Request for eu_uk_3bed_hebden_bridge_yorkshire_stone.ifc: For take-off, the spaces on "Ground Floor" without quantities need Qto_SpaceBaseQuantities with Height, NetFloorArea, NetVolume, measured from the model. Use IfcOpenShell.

First a look at what the model holds.

```python
import ifcopenshell
import ifcopenshell.util.element
import ifcopenshell.util.unit

model = ifcopenshell.open("eu_uk_3bed_hebden_bridge_yorkshire_stone.ifc")
print(model.schema)
for unit_type in ("LENGTHUNIT", "AREAUNIT", "VOLUMEUNIT"):
    print(unit_type, ifcopenshell.util.unit.calculate_unit_scale(model, unit_type))
storey = next(s for s in model.by_type("IfcBuildingStorey") if s.Name == "Ground Floor")
spaces = [e for e in ifcopenshell.util.element.get_decomposition(storey) if e.is_a("IfcSpace")]
for e in sorted(spaces, key=lambda e: e.id()):
    print(e.id(), e.is_a(), e.Name, list(ifcopenshell.util.element.get_psets(e, qtos_only=True)), sep=" | ")
```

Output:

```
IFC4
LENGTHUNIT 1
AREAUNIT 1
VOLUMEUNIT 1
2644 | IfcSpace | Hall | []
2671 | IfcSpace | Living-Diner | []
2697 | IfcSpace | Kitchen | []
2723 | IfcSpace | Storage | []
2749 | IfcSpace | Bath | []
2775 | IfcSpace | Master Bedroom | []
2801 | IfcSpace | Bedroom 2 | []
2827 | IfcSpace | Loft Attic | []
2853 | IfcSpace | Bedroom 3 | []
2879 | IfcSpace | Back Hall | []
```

```python
import ifcopenshell
import ifcopenshell.api.pset
import ifcopenshell.geom
import ifcopenshell.util.element
import ifcopenshell.util.shape
import ifcopenshell.util.unit

model = ifcopenshell.open("eu_uk_3bed_hebden_bridge_yorkshire_stone.ifc")
unit_scale = ifcopenshell.util.unit.calculate_unit_scale(model)
area_scale = ifcopenshell.util.unit.calculate_unit_scale(model, "AREAUNIT")
volume_scale = ifcopenshell.util.unit.calculate_unit_scale(model, "VOLUMEUNIT")
settings = ifcopenshell.geom.settings()

storey = next(s for s in model.by_type("IfcBuildingStorey") if s.Name == "Ground Floor")
spaces = [e for e in ifcopenshell.util.element.get_decomposition(storey) if e.is_a("IfcSpace")]

for e in sorted(spaces, key=lambda e: e.id()):
    if ifcopenshell.util.element.get_psets(e, qtos_only=True, should_inherit=False):
        continue
    # Geometry comes back in metres, in the element's own axes.
    shape = ifcopenshell.geom.create_shape(settings, e)
    values = {
        "Height": ifcopenshell.util.shape.get_z(shape.geometry) / unit_scale,
        "NetFloorArea": ifcopenshell.util.shape.get_footprint_area(shape.geometry) / area_scale,
        "NetVolume": ifcopenshell.util.shape.get_volume(shape.geometry) / volume_scale,
    }
    qto = ifcopenshell.api.pset.add_qto(model, product=e, name="Qto_SpaceBaseQuantities")
    ifcopenshell.api.pset.edit_qto(model, qto=qto, properties=values)
    print(e.id(), {k: round(v, 3) for k, v in values.items()})

model.write("eu_uk_3bed_hebden_bridge_yorkshire_stone_updated.ifc")
```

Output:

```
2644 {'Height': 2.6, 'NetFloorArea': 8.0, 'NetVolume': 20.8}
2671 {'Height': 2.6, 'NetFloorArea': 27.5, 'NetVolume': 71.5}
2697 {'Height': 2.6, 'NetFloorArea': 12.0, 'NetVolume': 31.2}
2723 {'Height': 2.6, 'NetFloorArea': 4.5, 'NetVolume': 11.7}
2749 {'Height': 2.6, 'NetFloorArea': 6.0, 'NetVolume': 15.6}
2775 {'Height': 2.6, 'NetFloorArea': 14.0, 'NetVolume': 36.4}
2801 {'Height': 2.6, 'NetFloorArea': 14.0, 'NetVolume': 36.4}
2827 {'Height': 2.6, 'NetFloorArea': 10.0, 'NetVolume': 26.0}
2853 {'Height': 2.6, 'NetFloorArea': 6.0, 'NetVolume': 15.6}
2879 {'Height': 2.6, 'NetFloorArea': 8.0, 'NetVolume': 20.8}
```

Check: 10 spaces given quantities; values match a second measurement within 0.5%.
